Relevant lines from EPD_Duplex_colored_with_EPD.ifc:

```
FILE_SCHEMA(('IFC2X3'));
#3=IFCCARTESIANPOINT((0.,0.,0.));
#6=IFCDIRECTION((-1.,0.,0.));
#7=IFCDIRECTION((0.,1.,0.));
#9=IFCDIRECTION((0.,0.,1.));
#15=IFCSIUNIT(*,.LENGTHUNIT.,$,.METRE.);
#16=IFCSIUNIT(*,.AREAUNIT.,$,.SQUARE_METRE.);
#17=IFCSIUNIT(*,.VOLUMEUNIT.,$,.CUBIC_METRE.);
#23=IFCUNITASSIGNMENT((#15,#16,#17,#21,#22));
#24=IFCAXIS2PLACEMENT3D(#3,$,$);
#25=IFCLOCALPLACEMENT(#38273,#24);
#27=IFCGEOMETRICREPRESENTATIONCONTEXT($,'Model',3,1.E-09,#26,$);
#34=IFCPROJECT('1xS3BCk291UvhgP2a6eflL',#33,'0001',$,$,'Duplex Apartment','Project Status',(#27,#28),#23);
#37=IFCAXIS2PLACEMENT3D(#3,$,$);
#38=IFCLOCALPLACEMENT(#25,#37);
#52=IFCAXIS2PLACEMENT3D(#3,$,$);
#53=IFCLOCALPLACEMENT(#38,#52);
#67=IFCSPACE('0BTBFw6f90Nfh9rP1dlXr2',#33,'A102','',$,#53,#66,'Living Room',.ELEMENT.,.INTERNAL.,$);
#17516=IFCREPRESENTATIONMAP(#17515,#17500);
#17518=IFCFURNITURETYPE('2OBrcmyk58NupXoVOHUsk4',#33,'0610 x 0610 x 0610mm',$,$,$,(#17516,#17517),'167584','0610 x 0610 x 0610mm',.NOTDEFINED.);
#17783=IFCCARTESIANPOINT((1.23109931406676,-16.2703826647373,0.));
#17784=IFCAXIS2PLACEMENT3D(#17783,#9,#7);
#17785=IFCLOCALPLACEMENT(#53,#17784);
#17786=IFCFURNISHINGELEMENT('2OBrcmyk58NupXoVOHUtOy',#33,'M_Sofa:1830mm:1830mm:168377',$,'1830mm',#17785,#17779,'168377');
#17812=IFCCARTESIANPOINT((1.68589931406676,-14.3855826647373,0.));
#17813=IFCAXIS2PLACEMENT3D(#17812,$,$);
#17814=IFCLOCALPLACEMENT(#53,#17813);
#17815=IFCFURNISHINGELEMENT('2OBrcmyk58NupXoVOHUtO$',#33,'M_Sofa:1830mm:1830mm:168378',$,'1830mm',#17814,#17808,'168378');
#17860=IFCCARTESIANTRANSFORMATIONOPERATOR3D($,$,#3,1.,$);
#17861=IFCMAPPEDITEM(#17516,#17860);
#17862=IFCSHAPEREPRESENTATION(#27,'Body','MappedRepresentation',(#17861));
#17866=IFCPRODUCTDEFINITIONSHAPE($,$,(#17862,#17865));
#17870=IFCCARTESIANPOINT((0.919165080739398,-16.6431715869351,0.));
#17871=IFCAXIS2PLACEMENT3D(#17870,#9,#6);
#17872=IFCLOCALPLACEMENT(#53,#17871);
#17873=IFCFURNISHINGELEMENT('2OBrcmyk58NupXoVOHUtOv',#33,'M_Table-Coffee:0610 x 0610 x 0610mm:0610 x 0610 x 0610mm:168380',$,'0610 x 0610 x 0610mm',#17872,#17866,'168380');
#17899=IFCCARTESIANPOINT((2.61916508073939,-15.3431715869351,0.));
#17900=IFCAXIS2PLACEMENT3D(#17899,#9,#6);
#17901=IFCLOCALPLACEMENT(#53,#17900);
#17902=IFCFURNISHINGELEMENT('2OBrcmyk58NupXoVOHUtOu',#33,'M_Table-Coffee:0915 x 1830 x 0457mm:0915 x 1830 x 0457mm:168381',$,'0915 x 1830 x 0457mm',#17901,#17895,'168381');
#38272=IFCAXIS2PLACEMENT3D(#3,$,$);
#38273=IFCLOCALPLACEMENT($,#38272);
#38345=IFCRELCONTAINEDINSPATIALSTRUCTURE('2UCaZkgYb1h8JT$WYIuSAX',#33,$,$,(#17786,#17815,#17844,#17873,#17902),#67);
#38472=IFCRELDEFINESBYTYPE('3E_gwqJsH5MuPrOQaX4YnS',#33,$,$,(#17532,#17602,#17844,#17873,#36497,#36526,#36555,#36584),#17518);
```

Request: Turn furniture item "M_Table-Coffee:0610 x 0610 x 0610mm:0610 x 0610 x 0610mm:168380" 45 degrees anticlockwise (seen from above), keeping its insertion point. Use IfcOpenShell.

```python
import ifcopenshell
import ifcopenshell.api.geometry
import ifcopenshell.util.placement

model = ifcopenshell.open("EPD_Duplex_colored_with_EPD.ifc")

item = model.by_guid("2OBrcmyk58NupXoVOHUtOv")
matrix = ifcopenshell.util.placement.get_local_placement(item.ObjectPlacement)
matrix = matrix @ ifcopenshell.util.placement.rotation(45, "Z")
ifcopenshell.api.geometry.edit_object_placement(model, product=item, matrix=matrix, is_si=False)

print(ifcopenshell.util.placement.get_local_placement(item.ObjectPlacement).round(3) + 0.0)

model.write("EPD_Duplex_colored_with_EPD_v2.ifc")
```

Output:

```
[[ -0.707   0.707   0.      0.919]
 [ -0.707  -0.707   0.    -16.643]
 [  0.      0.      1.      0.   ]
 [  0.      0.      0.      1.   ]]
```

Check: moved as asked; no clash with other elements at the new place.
